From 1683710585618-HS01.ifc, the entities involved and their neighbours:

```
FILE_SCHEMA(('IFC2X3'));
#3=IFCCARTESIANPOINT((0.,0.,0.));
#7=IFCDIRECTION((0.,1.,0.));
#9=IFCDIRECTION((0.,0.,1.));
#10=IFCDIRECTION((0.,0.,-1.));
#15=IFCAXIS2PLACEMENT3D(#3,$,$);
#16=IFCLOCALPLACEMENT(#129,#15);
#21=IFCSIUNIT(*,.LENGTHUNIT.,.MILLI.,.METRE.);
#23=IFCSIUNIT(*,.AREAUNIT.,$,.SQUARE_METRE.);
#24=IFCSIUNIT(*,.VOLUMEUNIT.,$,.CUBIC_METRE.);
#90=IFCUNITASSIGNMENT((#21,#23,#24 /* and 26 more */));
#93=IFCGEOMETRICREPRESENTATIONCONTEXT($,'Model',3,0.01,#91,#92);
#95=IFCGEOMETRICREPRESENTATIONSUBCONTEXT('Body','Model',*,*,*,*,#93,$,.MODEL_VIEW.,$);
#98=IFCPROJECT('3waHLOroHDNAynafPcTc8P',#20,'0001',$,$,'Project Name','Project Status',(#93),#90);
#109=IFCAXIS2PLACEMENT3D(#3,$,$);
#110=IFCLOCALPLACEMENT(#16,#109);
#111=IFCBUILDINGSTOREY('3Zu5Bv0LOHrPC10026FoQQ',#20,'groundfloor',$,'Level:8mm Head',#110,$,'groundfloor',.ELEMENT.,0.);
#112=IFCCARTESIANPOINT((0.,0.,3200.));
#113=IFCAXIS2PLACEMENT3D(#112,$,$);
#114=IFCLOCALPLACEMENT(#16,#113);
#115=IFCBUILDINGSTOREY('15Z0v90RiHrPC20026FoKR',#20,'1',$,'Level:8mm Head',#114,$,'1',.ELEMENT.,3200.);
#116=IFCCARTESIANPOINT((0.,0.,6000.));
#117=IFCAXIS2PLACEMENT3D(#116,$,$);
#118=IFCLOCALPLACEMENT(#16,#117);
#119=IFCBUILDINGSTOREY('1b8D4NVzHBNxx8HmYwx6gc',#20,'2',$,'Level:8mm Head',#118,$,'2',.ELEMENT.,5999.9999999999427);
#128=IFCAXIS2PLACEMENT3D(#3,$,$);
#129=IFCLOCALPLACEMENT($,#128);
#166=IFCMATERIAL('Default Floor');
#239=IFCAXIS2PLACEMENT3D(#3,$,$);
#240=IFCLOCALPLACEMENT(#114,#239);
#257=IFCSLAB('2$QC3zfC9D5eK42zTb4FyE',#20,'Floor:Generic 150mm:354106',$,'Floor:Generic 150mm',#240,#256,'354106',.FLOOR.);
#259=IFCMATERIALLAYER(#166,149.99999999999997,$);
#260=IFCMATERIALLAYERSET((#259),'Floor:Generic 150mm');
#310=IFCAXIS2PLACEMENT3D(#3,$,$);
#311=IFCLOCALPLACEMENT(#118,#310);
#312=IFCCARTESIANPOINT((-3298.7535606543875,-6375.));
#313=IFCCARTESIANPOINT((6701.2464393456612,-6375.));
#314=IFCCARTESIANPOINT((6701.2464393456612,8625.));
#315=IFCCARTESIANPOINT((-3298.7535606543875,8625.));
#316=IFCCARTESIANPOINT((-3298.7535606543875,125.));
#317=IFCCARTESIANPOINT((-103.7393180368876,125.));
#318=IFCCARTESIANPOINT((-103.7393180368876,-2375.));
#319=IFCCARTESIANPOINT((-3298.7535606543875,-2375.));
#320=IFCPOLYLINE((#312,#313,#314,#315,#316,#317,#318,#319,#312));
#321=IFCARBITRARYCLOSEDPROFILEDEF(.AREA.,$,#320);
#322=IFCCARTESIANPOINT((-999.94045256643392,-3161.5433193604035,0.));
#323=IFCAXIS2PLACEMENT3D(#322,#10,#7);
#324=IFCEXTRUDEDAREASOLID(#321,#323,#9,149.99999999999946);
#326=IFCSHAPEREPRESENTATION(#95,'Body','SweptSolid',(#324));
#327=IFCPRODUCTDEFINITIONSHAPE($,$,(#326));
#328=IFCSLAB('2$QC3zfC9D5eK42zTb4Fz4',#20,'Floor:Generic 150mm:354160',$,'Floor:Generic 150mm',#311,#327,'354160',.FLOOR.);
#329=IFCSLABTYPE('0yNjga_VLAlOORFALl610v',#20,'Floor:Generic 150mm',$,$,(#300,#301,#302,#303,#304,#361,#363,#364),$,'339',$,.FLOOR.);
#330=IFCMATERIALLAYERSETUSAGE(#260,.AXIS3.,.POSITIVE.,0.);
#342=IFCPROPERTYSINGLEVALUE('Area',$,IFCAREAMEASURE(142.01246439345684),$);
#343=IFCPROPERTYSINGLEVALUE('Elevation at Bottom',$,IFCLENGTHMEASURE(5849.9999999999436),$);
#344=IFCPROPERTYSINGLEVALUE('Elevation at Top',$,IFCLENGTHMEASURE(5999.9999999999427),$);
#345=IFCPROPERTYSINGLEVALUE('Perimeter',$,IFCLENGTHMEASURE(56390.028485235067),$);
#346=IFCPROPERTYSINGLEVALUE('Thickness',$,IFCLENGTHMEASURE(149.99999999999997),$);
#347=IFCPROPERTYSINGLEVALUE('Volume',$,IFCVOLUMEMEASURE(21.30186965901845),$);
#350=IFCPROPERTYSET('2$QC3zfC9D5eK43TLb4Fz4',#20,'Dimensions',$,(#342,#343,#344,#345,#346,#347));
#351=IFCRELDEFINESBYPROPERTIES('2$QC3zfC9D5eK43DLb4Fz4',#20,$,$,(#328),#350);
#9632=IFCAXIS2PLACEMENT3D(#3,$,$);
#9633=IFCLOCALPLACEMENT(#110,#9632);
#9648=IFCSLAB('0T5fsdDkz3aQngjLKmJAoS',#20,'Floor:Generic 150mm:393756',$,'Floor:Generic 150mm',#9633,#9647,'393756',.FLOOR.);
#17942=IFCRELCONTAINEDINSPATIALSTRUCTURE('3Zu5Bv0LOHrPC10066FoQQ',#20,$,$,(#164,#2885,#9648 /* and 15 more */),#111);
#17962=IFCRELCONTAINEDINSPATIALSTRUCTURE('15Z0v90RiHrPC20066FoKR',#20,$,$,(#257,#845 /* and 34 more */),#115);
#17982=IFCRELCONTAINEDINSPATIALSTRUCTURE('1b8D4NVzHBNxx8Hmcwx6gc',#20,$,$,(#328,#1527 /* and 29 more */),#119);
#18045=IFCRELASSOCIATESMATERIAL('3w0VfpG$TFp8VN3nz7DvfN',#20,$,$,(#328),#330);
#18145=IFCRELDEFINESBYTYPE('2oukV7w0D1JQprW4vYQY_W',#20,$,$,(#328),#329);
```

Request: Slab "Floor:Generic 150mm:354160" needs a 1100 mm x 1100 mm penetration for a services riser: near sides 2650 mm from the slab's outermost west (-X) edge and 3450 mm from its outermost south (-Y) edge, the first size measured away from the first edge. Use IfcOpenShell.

```python
import numpy as np
import ifcopenshell
import ifcopenshell.api.feature
import ifcopenshell.api.geometry
import ifcopenshell.api.pset
import ifcopenshell.api.root
import ifcopenshell.geom
import ifcopenshell.util.element
import ifcopenshell.util.placement
import ifcopenshell.util.representation
import ifcopenshell.util.shape
import ifcopenshell.util.unit

model = ifcopenshell.open("1683710585618-HS01.ifc")
unit_scale = ifcopenshell.util.unit.calculate_unit_scale(model)
area_scale = ifcopenshell.util.unit.calculate_unit_scale(model, "AREAUNIT")
volume_scale = ifcopenshell.util.unit.calculate_unit_scale(model, "VOLUMEUNIT")
settings = ifcopenshell.geom.settings()


def volume(element):
    """Net volume in cubic metres, openings subtracted."""
    shape = ifcopenshell.geom.create_shape(settings, element)
    return ifcopenshell.util.shape.get_volume(shape.geometry)


slab = model.by_guid("2$QC3zfC9D5eK42zTb4Fz4")
before = volume(slab)

# Extent in the slab's own axes, in metres. The edges named are its -X and -Y sides.
slab_shape = ifcopenshell.geom.create_shape(settings, slab)
vertices = ifcopenshell.util.shape.get_vertices(slab_shape.geometry)
x_min, y_min, bottom = vertices.min(axis=0)
top = vertices[:, 2].max()

opening = ifcopenshell.api.root.create_entity(model, ifc_class="IfcOpeningElement", name="Services riser opening")
context = ifcopenshell.util.representation.get_context(model, "Model", "Body", "MODEL_VIEW")
width, depth = 1.1, 1.1
outline = [(0.0, 0.0), (width, 0.0), (width, depth), (0.0, depth), (0.0, 0.0)]
# Overshoot both faces by 50 mm so the cut is clean.
shape = ifcopenshell.api.geometry.add_slab_representation(
    model, context=context, depth=top - bottom + 0.1, polyline=outline
)
ifcopenshell.api.geometry.assign_representation(model, product=opening, representation=shape)

matrix = ifcopenshell.util.placement.get_local_placement(slab.ObjectPlacement)
matrix[:, 3] = matrix @ np.append(np.array([x_min + 2.65, y_min + 3.45, bottom - 0.05]) / unit_scale, 1.0)
ifcopenshell.api.geometry.edit_object_placement(model, product=opening, matrix=matrix, is_si=False)
ifcopenshell.api.feature.add_feature(model, feature=opening, element=slab)

after = volume(slab)

# Update the slab's stored quantities.
pset = model.by_id(ifcopenshell.util.element.get_pset(slab, "Dimensions", should_inherit=False)["id"])
ifcopenshell.api.pset.edit_pset(model, pset=pset, properties={
    "Area": model.create_entity("IfcAreaMeasure", after / (top - bottom) / area_scale),
    "Volume": model.create_entity("IfcVolumeMeasure", after / volume_scale),
})

print(f"slab volume {before:.3f} -> {after:.3f} m3")

model.write("1683710585618-HS01-out.ifc")
```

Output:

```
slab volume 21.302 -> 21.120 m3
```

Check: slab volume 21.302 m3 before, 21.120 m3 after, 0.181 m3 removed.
